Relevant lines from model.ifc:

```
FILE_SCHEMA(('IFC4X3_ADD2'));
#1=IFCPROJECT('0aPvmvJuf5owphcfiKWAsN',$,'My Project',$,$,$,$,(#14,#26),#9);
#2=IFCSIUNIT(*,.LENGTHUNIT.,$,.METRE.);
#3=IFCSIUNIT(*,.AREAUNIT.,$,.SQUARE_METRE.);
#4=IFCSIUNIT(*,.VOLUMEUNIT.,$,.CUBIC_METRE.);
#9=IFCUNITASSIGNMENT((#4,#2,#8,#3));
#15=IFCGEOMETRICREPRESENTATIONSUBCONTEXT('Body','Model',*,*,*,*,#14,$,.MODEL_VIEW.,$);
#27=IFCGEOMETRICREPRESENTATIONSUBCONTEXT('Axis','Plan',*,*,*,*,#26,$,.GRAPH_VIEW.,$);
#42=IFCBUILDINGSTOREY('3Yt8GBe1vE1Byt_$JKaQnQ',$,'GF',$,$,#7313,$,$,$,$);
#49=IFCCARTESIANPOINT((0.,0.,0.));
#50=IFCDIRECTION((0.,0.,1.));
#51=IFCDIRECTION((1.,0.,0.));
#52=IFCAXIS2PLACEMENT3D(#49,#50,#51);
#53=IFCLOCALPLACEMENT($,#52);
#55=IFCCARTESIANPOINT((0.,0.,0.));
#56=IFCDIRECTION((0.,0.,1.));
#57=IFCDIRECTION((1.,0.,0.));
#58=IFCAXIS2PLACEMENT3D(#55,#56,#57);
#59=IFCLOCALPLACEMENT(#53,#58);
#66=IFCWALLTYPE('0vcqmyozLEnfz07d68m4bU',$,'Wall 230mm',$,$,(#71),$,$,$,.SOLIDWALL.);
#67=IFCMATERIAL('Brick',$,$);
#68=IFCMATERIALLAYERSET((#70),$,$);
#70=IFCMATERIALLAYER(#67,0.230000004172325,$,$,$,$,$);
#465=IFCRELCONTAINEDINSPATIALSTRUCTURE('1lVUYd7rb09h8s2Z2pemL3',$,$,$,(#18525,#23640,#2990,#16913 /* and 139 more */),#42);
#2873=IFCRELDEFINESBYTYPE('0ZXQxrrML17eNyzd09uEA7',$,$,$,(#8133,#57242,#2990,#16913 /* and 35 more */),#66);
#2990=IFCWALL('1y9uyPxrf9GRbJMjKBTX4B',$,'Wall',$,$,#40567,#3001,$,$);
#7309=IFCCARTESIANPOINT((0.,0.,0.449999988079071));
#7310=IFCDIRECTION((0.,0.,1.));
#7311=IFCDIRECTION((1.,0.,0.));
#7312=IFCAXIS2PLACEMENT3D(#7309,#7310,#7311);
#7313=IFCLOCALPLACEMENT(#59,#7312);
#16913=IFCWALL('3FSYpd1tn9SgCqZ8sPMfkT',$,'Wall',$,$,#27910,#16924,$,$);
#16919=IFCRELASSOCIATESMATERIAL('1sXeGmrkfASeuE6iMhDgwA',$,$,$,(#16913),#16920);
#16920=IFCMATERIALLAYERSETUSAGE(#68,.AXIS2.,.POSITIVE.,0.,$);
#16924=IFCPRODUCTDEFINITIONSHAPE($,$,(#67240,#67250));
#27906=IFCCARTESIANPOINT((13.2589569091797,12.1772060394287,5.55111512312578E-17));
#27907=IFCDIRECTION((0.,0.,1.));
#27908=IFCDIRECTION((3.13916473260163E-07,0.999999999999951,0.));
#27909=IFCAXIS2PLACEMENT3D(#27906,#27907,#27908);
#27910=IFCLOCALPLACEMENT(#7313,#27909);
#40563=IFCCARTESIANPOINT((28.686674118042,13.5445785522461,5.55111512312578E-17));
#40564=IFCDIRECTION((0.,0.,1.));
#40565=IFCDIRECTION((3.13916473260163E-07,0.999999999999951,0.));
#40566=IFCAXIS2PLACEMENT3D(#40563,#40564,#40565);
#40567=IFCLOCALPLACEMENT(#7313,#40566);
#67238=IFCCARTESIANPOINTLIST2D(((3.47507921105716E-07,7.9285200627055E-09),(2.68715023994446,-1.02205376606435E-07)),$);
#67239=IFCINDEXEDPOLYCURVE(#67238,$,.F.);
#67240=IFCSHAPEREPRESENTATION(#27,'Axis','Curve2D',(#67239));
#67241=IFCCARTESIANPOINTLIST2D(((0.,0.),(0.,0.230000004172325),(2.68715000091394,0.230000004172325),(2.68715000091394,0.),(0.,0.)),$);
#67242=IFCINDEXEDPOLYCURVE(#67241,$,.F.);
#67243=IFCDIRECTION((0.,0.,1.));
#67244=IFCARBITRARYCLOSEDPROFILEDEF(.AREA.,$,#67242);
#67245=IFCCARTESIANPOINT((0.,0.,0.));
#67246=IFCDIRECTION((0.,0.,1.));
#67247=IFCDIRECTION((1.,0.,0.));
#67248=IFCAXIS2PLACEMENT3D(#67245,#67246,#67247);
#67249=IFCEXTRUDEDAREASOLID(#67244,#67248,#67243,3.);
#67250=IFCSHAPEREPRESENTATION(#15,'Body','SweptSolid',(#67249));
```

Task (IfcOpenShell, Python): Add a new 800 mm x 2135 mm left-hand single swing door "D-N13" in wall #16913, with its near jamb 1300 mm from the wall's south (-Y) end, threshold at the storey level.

```python
import numpy as np
import ifcopenshell
import ifcopenshell.api.feature
import ifcopenshell.api.geometry
import ifcopenshell.api.root
import ifcopenshell.api.spatial
import ifcopenshell.geom
import ifcopenshell.util.element
import ifcopenshell.util.placement
import ifcopenshell.util.representation
import ifcopenshell.util.shape
import ifcopenshell.util.unit

model = ifcopenshell.open("model.ifc")
unit_scale = ifcopenshell.util.unit.calculate_unit_scale(model)
settings = ifcopenshell.geom.settings()


def volume(element):
    """Net volume in cubic metres, openings subtracted."""
    shape = ifcopenshell.geom.create_shape(settings, element)
    return ifcopenshell.util.shape.get_volume(shape.geometry)


wall = model.by_guid("3FSYpd1tn9SgCqZ8sPMfkT")
storey = ifcopenshell.util.element.get_container(wall, ifc_class="IfcBuildingStorey")
context = ifcopenshell.util.representation.get_context(model, "Model", "Body", "MODEL_VIEW")
before = volume(wall)

width, height, from_end, sill = 0.8, 2.135, 1.3, 0.0  # metres

# The wall runs along its own X axis, and the end named is its -X end.
wall_shape = ifcopenshell.geom.create_shape(settings, wall)
x, y, z = ifcopenshell.util.shape.get_vertices(wall_shape.geometry).T
start = x.min() + from_end
face, thickness = float(y.min()), float(y.max() - y.min())
wall_matrix = ifcopenshell.util.placement.get_local_placement(wall.ObjectPlacement)
level = ifcopenshell.util.placement.get_local_placement(storey.ObjectPlacement)[2, 3]


def in_wall(x, y):
    """Placement at x, y metres in the wall's axes, at sill height."""
    matrix = wall_matrix.copy()
    matrix[:, 3] = wall_matrix @ np.array([x / unit_scale, y / unit_scale, 0.0, 1.0])
    matrix[2, 3] = level + sill / unit_scale
    return matrix


# Opening: a box that overshoots both wall faces by 50 mm.
opening = ifcopenshell.api.root.create_entity(model, ifc_class="IfcOpeningElement", predefined_type="OPENING")
box = ifcopenshell.api.geometry.add_wall_representation(
    model, context=context, length=width, height=height, thickness=thickness + 0.1
)
ifcopenshell.api.geometry.assign_representation(model, product=opening, representation=box)
ifcopenshell.api.geometry.edit_object_placement(model, product=opening, matrix=in_wall(start, face - 0.05), is_si=False)
ifcopenshell.api.feature.add_feature(model, feature=opening, element=wall)

door = ifcopenshell.api.root.create_entity(model, ifc_class="IfcDoor", name="D-N13", predefined_type="DOOR")
door.OverallWidth, door.OverallHeight = width / unit_scale, height / unit_scale
door.OperationType = "SINGLE_SWING_LEFT"
body = ifcopenshell.api.geometry.add_door_representation(
    model,
    context=context,
    overall_width=door.OverallWidth,
    overall_height=door.OverallHeight,
    operation_type="SINGLE_SWING_LEFT",
    lining_properties={"LiningDepth": thickness / unit_scale, "ThresholdDepth": thickness / unit_scale},
)
ifcopenshell.api.geometry.assign_representation(model, product=door, representation=body)
ifcopenshell.api.spatial.assign_container(model, products=[door], relating_structure=storey)
ifcopenshell.api.feature.add_filling(model, opening=opening, element=door)

# The lining spans the wall, so the door starts at the wall face.
ifcopenshell.api.geometry.edit_object_placement(model, product=door, matrix=in_wall(start, face), is_si=False)

after = volume(wall)

print(f"wall volume {before:.3f} -> {after:.3f} m3")

model.write("model_updated.ifc")
```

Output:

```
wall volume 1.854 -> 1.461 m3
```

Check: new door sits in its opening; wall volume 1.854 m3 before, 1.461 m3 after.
